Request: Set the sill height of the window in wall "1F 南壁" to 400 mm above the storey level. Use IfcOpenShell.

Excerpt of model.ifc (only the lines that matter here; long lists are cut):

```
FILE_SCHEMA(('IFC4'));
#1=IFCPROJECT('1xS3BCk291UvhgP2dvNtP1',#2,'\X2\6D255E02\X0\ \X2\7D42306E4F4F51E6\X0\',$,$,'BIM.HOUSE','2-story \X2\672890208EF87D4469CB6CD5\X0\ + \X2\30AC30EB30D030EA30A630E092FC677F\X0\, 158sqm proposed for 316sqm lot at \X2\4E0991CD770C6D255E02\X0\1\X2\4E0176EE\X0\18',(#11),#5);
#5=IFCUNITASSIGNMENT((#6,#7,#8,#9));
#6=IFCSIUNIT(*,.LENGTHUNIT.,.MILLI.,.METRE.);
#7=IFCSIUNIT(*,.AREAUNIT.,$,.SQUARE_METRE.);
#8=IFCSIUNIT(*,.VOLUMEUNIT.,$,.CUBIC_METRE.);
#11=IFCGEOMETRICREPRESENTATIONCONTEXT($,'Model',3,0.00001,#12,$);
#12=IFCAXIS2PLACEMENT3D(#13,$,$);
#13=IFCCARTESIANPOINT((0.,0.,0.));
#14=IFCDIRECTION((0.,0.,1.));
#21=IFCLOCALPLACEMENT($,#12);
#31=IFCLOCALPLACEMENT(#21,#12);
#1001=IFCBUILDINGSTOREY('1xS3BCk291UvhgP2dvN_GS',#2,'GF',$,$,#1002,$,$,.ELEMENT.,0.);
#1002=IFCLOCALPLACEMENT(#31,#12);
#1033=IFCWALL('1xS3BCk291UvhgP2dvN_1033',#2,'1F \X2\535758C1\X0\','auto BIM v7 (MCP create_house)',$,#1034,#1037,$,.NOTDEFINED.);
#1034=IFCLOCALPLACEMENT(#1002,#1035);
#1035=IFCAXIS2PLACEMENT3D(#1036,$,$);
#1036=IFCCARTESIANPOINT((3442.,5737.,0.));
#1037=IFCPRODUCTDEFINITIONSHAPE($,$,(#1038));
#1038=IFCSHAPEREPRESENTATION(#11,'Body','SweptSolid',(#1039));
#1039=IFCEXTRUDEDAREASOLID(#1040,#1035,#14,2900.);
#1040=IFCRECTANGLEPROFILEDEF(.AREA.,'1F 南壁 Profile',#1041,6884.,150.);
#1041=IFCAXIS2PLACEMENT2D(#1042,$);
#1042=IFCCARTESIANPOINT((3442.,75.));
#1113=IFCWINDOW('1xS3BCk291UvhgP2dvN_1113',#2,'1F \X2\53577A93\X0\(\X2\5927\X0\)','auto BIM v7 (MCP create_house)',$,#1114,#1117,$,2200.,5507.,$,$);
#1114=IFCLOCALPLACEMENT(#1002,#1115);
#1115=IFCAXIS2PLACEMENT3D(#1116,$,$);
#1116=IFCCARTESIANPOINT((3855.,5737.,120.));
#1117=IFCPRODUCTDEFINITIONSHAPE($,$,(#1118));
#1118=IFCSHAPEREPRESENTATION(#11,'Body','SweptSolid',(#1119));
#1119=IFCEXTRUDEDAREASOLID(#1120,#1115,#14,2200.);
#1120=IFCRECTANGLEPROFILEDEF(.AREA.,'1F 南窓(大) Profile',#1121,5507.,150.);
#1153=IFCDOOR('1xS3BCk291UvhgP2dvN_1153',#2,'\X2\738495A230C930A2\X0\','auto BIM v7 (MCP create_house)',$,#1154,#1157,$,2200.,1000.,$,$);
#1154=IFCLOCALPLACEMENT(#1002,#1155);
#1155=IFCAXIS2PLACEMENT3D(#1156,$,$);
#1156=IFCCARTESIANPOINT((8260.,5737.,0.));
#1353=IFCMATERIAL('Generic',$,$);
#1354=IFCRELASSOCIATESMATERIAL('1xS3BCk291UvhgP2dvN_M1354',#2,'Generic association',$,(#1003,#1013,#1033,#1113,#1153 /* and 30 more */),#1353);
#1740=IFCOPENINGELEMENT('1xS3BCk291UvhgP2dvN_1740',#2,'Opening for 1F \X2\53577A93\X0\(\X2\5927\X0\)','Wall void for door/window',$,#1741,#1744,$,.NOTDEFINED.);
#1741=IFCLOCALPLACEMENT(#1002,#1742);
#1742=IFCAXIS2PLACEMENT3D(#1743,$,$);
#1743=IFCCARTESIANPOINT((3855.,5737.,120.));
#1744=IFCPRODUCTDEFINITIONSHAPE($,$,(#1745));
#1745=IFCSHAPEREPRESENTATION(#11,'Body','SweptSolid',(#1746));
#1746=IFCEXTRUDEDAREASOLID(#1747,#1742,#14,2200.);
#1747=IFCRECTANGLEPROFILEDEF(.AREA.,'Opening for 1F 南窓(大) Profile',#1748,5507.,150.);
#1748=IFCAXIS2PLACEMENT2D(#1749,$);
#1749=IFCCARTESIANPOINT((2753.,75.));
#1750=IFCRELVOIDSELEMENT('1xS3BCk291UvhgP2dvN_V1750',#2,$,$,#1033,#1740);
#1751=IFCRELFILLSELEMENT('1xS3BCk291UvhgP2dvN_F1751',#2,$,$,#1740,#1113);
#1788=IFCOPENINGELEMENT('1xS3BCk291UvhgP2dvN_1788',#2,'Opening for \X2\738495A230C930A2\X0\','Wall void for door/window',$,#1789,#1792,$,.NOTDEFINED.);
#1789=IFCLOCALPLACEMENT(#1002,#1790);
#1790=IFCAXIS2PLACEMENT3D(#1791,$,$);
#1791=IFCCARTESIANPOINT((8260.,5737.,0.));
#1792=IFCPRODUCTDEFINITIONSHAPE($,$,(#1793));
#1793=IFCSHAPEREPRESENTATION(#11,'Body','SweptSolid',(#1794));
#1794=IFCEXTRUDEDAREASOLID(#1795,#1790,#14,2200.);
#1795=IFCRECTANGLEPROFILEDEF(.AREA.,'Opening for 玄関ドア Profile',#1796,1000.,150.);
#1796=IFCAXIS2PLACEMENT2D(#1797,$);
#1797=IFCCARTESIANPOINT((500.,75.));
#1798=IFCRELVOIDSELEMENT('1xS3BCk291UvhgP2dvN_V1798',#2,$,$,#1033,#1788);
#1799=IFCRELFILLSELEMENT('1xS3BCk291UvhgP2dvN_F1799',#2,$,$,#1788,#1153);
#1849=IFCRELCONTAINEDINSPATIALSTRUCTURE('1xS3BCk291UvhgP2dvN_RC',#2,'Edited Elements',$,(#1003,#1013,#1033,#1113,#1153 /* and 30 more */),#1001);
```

```python
import numpy as np
import ifcopenshell
import ifcopenshell.api.geometry
import ifcopenshell.geom
import ifcopenshell.util.element
import ifcopenshell.util.placement
import ifcopenshell.util.shape
import ifcopenshell.util.unit

model = ifcopenshell.open("model.ifc")
unit_scale = ifcopenshell.util.unit.calculate_unit_scale(model)

window = model.by_guid("1xS3BCk291UvhgP2dvN_1113")
opening = window.FillsVoids[0].RelatingOpeningElement
storey = ifcopenshell.util.element.get_container(window, ifc_class="IfcBuildingStorey")
level = ifcopenshell.util.placement.get_local_placement(storey.ObjectPlacement)[2, 3]

# The opening's origin need not be at the sill, so measure its lowest point.
shape = ifcopenshell.geom.create_shape(ifcopenshell.geom.settings(), opening)
bottom = ifcopenshell.util.shape.get_shape_bottom_elevation(shape, shape.geometry) / unit_scale
dz = level + 0.4 / unit_scale - bottom

shift = np.array([0.0, 0.0, dz])
# The window is not placed relative to its opening, so move both.
for product in (opening, window):
    matrix = ifcopenshell.util.placement.get_local_placement(product.ObjectPlacement)
    matrix[:3, 3] += shift
    ifcopenshell.api.geometry.edit_object_placement(model, product=product, matrix=matrix, is_si=False)

print(f"moved by {dz * unit_scale:+.3f} m")

model.write("model_edited.ifc")
```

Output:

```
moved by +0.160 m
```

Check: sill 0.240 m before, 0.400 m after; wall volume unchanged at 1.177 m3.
